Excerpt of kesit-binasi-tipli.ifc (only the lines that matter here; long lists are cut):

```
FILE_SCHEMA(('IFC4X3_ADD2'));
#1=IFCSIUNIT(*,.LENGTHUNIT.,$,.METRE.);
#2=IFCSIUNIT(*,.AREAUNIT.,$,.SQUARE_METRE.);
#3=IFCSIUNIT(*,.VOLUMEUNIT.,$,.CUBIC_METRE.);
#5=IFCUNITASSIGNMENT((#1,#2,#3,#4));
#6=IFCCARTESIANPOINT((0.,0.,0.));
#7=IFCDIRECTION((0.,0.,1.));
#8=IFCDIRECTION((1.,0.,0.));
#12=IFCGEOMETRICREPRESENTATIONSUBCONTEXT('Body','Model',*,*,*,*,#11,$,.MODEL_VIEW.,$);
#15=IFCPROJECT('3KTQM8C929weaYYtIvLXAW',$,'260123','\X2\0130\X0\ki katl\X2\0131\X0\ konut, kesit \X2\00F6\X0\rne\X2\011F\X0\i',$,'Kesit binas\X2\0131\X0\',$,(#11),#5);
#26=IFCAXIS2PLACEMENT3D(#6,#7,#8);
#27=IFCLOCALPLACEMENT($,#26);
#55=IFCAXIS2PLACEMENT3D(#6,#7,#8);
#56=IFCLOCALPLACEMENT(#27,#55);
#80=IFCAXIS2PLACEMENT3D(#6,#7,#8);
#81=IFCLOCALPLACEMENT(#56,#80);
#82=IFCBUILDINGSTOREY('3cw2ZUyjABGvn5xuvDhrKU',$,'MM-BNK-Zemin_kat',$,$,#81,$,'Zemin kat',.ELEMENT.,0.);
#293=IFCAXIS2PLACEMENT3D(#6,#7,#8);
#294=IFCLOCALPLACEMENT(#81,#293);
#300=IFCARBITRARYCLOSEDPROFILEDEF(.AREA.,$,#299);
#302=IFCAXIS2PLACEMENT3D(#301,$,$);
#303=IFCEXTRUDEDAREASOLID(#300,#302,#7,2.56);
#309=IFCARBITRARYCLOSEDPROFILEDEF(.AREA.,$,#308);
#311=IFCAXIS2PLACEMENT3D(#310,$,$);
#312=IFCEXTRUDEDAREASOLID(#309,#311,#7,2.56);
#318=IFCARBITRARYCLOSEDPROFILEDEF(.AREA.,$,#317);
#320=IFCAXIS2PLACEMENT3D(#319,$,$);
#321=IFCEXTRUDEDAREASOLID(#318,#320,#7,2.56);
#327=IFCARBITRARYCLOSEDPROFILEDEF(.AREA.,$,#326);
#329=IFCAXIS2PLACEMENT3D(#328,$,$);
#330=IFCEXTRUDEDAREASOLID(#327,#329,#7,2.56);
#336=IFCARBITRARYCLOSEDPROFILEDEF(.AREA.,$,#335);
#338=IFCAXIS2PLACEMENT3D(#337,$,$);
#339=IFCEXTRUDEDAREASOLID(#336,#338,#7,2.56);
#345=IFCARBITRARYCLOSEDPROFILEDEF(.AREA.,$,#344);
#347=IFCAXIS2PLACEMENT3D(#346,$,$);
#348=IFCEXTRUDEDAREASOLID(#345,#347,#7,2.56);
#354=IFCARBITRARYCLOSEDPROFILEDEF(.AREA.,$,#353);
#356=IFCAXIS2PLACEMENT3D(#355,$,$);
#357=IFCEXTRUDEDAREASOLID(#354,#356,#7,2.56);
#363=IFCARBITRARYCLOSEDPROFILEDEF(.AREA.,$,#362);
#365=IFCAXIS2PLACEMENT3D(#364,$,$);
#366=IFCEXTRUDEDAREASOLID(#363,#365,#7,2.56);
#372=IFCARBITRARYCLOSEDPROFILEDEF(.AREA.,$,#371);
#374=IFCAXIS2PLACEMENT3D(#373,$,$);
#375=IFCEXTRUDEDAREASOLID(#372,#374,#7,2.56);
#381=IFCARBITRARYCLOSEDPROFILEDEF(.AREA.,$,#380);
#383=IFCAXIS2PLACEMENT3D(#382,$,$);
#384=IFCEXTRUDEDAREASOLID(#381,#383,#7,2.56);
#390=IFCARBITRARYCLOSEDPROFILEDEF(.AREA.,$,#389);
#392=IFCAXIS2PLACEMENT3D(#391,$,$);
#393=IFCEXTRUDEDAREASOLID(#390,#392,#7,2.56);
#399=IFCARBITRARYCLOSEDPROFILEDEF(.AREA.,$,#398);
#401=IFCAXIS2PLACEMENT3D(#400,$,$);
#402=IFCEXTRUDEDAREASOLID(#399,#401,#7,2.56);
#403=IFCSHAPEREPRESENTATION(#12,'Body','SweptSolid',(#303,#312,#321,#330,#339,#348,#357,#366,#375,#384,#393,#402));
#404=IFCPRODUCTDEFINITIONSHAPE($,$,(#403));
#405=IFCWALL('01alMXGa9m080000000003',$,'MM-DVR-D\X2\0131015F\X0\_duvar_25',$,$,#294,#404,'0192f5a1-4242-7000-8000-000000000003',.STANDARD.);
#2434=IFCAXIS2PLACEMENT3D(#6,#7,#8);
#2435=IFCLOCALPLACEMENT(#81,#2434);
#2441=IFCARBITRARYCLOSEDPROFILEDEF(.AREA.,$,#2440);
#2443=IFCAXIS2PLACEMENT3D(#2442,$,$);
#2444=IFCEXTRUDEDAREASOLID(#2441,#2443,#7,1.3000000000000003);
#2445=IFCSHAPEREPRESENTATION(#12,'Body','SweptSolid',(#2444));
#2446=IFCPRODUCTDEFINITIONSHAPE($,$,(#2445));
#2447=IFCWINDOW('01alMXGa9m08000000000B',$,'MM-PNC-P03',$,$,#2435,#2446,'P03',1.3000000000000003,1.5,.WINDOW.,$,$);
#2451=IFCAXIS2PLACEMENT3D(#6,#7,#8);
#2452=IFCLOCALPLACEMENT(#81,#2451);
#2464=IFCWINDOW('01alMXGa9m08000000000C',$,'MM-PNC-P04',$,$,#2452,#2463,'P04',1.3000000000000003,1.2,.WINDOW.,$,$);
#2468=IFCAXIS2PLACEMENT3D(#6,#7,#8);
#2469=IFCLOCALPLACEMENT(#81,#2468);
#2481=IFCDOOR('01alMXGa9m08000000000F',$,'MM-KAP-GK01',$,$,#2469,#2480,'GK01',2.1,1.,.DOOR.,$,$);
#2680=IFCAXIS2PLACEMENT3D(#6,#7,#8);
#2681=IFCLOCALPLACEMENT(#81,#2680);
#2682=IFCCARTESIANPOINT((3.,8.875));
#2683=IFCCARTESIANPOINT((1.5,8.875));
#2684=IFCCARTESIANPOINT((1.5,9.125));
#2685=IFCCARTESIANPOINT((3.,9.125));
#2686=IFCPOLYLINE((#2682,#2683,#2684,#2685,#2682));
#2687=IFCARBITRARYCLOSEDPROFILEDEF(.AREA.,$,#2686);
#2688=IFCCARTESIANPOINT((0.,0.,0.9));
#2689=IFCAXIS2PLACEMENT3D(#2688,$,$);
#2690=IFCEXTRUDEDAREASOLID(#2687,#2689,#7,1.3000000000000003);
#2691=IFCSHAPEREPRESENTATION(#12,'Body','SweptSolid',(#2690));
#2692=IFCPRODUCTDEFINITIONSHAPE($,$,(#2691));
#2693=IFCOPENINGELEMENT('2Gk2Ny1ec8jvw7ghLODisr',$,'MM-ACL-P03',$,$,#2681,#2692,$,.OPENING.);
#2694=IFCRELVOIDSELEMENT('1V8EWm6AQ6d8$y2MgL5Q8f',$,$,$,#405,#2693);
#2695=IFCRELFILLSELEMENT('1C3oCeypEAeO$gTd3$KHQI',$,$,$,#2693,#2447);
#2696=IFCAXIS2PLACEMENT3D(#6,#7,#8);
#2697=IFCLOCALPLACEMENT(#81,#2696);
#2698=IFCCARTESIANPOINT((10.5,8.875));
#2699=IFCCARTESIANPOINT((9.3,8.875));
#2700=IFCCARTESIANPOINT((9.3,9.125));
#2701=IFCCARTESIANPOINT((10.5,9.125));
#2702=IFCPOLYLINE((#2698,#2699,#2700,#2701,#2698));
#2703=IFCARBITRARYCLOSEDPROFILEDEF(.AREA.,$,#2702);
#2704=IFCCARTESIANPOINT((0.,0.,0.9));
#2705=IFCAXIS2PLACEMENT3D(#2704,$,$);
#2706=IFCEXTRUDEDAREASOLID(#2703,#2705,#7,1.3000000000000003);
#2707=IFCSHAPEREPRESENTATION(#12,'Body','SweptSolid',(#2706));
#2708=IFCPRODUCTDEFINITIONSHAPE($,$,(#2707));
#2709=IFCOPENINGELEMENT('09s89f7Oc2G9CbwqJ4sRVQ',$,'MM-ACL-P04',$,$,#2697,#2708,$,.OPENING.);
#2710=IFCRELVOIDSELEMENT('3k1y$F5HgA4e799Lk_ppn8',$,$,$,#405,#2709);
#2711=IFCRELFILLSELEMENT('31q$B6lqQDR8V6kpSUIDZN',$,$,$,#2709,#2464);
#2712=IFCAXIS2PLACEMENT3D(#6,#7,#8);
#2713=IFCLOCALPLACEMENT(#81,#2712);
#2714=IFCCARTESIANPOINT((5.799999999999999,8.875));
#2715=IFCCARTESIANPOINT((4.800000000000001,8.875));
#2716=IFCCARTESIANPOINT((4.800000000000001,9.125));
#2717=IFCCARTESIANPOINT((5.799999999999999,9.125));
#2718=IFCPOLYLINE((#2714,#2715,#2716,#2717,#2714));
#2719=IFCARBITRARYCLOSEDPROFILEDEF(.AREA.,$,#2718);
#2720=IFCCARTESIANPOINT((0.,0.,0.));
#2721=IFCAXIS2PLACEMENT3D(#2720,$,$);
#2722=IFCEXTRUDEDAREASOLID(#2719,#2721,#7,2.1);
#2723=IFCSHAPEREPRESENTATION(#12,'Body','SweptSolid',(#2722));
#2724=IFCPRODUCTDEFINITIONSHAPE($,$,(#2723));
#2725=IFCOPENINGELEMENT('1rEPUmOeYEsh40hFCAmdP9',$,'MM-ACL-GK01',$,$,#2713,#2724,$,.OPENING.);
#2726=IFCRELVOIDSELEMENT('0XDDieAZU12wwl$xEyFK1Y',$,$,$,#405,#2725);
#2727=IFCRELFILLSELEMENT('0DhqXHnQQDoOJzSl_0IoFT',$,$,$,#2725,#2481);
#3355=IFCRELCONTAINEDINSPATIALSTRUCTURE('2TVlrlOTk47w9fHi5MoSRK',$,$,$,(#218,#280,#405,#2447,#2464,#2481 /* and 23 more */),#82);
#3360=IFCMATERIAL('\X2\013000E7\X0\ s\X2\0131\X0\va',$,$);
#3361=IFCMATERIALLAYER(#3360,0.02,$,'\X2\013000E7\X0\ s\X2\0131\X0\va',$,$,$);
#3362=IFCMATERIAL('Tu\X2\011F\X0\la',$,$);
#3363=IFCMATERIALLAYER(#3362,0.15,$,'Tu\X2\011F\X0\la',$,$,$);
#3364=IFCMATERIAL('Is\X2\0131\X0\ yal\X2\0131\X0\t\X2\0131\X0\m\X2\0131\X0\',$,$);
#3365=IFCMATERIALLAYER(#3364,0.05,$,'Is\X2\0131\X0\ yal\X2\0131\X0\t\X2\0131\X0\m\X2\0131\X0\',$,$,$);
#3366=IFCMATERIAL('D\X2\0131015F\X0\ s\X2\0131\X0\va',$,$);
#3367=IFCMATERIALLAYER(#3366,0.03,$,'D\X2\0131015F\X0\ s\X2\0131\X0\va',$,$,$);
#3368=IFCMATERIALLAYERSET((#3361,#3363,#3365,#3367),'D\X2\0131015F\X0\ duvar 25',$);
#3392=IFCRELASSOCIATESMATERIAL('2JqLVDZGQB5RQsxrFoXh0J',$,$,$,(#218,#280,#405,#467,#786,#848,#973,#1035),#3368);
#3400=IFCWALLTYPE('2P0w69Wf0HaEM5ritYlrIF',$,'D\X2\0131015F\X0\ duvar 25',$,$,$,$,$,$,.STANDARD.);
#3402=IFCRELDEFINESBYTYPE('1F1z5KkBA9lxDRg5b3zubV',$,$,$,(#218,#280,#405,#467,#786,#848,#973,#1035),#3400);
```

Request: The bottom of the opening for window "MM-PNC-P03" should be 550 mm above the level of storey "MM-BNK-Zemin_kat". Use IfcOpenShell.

```python
import numpy as np
import ifcopenshell
import ifcopenshell.api.geometry
import ifcopenshell.geom
import ifcopenshell.util.element
import ifcopenshell.util.placement
import ifcopenshell.util.shape
import ifcopenshell.util.unit

model = ifcopenshell.open("kesit-binasi-tipli.ifc")
unit_scale = ifcopenshell.util.unit.calculate_unit_scale(model)

window = model.by_guid("01alMXGa9m08000000000B")
opening = window.FillsVoids[0].RelatingOpeningElement
storey = ifcopenshell.util.element.get_container(window, ifc_class="IfcBuildingStorey")
level = ifcopenshell.util.placement.get_local_placement(storey.ObjectPlacement)[2, 3]

# The opening's origin need not be at the sill, so measure its lowest point.
shape = ifcopenshell.geom.create_shape(ifcopenshell.geom.settings(), opening)
bottom = ifcopenshell.util.shape.get_shape_bottom_elevation(shape, shape.geometry) / unit_scale
dz = level + 0.55 / unit_scale - bottom

shift = np.array([0.0, 0.0, dz])
# The window is not placed relative to its opening, so move both.
for product in (opening, window):
    matrix = ifcopenshell.util.placement.get_local_placement(product.ObjectPlacement)
    matrix[:3, 3] += shift
    ifcopenshell.api.geometry.edit_object_placement(model, product=product, matrix=matrix, is_si=False)

print(f"moved by {dz * unit_scale:+.3f} m")

model.write("kesit-binasi-tipli_rev.ifc")
```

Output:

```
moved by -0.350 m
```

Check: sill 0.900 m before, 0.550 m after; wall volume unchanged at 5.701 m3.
